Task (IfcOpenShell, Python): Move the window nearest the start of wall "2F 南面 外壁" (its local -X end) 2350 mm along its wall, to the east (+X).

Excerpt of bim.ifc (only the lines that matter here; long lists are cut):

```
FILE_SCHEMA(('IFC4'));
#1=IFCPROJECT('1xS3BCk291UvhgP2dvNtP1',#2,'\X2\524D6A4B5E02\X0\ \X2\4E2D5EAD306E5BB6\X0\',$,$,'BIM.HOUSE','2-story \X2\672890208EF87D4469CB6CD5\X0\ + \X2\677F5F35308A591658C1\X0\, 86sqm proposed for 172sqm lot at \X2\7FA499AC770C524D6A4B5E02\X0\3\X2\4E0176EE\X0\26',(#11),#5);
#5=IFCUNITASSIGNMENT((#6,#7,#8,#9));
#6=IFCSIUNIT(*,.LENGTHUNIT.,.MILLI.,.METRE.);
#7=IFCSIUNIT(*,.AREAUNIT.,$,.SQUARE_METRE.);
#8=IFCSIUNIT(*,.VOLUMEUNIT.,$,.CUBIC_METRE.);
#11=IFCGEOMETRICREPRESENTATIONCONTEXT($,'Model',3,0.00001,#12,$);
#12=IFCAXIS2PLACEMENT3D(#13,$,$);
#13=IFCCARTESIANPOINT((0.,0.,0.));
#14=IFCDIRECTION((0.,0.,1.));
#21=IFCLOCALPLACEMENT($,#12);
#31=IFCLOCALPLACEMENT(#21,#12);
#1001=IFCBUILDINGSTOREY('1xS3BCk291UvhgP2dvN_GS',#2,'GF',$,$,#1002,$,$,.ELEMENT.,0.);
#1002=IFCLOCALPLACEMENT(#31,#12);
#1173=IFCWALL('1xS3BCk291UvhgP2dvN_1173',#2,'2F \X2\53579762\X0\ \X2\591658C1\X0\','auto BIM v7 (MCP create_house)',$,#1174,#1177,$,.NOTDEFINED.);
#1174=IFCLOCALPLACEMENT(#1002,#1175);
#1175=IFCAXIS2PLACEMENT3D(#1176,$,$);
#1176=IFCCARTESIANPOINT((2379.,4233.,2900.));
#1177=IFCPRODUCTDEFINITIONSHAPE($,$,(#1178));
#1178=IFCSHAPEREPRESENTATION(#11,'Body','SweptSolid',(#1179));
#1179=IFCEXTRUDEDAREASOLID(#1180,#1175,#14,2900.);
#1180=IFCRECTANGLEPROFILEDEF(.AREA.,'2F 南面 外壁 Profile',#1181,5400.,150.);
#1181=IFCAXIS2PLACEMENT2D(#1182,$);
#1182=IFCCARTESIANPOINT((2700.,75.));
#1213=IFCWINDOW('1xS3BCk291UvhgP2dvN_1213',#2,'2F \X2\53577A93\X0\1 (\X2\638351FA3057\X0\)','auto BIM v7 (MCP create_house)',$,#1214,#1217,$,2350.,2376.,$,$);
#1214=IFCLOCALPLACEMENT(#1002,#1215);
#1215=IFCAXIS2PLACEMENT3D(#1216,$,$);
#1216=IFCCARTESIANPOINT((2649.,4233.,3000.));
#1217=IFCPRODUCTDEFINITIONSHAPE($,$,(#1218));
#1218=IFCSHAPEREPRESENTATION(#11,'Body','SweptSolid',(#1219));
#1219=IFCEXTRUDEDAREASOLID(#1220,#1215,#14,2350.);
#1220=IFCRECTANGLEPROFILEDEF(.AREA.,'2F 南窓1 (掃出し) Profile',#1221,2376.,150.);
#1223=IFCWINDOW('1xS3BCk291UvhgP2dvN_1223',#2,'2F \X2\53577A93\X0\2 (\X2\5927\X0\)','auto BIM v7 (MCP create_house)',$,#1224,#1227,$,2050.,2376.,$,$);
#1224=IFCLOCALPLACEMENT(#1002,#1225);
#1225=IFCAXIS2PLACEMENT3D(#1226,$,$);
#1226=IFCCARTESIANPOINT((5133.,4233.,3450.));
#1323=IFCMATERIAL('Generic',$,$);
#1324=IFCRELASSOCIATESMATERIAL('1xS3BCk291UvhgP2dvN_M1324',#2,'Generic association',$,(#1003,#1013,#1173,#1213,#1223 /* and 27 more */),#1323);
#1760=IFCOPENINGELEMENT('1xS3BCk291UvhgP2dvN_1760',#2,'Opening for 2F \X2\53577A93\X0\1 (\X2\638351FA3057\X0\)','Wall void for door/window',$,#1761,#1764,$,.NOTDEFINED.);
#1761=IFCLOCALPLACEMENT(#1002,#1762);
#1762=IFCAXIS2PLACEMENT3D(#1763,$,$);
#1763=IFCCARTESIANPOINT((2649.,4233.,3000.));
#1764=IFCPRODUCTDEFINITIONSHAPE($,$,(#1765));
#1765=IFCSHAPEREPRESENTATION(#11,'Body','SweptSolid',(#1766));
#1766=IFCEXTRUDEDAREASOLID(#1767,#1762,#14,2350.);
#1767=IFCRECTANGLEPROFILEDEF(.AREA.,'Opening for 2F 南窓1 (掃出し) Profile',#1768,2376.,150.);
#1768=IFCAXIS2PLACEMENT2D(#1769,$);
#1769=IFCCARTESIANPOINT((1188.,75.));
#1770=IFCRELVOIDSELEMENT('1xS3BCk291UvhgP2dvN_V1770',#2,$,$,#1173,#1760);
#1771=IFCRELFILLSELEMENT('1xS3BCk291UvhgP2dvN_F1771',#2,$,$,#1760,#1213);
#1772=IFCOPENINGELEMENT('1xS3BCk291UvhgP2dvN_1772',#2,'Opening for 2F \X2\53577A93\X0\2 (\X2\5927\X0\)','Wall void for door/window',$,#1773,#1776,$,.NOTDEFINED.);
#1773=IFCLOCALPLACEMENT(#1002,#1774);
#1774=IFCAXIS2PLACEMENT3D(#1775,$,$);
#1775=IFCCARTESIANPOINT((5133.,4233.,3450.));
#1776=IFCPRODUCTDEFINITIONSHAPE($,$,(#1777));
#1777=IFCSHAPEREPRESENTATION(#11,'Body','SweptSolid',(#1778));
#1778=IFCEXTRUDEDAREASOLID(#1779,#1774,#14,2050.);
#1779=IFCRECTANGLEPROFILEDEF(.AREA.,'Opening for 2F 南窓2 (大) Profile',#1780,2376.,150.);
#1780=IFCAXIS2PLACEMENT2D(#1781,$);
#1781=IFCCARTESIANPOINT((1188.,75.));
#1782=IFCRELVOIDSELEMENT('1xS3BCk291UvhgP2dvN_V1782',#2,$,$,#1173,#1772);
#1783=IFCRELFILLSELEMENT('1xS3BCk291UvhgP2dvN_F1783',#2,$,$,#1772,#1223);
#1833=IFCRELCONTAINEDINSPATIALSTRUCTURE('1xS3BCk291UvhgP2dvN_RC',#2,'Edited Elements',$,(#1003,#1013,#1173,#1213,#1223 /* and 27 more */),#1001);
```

```python
import ifcopenshell
import ifcopenshell.api.geometry
import ifcopenshell.util.placement

model = ifcopenshell.open("bim.ifc")

window = model.by_guid("1xS3BCk291UvhgP2dvN_1213")
opening = window.FillsVoids[0].RelatingOpeningElement
wall = opening.VoidsElements[0].RelatingBuildingElement

wall_matrix = ifcopenshell.util.placement.get_local_placement(wall.ObjectPlacement)
shift = wall_matrix[:3, 0] * 2350.0
before = ifcopenshell.util.placement.get_local_placement(window.ObjectPlacement)[:3, 3].copy()

# The window is not placed relative to its opening, so move both.
for product in (opening, window):
    matrix = ifcopenshell.util.placement.get_local_placement(product.ObjectPlacement)
    matrix[:3, 3] += shift
    ifcopenshell.api.geometry.edit_object_placement(model, product=product, matrix=matrix, is_si=False)

after = ifcopenshell.util.placement.get_local_placement(window.ObjectPlacement)[:3, 3]
print("window moved by", (after - before).round(3) + 0.0)

model.write("bim-out.ifc")
```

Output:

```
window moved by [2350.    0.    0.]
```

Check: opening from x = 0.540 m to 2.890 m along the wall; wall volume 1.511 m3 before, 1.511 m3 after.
